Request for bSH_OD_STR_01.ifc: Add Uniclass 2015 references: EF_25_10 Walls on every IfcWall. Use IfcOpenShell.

First a look at what the model holds.

```python
import ifcopenshell

model = ifcopenshell.open("bSH_OD_STR_01.ifc")
print(model.schema)
print("classifications:", [c.Name for c in model.by_type("IfcClassification")])
for ifc_class in ("IfcDoor", "IfcRoof", "IfcStair", "IfcWall", "IfcWindow"):
    print(ifc_class, len(model.by_type(ifc_class)))
```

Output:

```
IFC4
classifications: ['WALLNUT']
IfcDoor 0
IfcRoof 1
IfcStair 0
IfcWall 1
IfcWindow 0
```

```python
import ifcopenshell
import ifcopenshell.api.classification

model = ifcopenshell.open("bSH_OD_STR_01.ifc")

system = ifcopenshell.api.classification.add_classification(model, classification="Uniclass 2015")

codes = {
    "IfcWall": ("EF_25_10", "Walls"),
}
for ifc_class, (code, name) in codes.items():
    products = model.by_type(ifc_class)
    ifcopenshell.api.classification.add_reference(
        model, products=products, classification=system, identification=code, name=name
    )
    print(code, len(products))

model.write("bSH_OD_STR_01_v2.ifc")
```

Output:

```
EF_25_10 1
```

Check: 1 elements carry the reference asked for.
